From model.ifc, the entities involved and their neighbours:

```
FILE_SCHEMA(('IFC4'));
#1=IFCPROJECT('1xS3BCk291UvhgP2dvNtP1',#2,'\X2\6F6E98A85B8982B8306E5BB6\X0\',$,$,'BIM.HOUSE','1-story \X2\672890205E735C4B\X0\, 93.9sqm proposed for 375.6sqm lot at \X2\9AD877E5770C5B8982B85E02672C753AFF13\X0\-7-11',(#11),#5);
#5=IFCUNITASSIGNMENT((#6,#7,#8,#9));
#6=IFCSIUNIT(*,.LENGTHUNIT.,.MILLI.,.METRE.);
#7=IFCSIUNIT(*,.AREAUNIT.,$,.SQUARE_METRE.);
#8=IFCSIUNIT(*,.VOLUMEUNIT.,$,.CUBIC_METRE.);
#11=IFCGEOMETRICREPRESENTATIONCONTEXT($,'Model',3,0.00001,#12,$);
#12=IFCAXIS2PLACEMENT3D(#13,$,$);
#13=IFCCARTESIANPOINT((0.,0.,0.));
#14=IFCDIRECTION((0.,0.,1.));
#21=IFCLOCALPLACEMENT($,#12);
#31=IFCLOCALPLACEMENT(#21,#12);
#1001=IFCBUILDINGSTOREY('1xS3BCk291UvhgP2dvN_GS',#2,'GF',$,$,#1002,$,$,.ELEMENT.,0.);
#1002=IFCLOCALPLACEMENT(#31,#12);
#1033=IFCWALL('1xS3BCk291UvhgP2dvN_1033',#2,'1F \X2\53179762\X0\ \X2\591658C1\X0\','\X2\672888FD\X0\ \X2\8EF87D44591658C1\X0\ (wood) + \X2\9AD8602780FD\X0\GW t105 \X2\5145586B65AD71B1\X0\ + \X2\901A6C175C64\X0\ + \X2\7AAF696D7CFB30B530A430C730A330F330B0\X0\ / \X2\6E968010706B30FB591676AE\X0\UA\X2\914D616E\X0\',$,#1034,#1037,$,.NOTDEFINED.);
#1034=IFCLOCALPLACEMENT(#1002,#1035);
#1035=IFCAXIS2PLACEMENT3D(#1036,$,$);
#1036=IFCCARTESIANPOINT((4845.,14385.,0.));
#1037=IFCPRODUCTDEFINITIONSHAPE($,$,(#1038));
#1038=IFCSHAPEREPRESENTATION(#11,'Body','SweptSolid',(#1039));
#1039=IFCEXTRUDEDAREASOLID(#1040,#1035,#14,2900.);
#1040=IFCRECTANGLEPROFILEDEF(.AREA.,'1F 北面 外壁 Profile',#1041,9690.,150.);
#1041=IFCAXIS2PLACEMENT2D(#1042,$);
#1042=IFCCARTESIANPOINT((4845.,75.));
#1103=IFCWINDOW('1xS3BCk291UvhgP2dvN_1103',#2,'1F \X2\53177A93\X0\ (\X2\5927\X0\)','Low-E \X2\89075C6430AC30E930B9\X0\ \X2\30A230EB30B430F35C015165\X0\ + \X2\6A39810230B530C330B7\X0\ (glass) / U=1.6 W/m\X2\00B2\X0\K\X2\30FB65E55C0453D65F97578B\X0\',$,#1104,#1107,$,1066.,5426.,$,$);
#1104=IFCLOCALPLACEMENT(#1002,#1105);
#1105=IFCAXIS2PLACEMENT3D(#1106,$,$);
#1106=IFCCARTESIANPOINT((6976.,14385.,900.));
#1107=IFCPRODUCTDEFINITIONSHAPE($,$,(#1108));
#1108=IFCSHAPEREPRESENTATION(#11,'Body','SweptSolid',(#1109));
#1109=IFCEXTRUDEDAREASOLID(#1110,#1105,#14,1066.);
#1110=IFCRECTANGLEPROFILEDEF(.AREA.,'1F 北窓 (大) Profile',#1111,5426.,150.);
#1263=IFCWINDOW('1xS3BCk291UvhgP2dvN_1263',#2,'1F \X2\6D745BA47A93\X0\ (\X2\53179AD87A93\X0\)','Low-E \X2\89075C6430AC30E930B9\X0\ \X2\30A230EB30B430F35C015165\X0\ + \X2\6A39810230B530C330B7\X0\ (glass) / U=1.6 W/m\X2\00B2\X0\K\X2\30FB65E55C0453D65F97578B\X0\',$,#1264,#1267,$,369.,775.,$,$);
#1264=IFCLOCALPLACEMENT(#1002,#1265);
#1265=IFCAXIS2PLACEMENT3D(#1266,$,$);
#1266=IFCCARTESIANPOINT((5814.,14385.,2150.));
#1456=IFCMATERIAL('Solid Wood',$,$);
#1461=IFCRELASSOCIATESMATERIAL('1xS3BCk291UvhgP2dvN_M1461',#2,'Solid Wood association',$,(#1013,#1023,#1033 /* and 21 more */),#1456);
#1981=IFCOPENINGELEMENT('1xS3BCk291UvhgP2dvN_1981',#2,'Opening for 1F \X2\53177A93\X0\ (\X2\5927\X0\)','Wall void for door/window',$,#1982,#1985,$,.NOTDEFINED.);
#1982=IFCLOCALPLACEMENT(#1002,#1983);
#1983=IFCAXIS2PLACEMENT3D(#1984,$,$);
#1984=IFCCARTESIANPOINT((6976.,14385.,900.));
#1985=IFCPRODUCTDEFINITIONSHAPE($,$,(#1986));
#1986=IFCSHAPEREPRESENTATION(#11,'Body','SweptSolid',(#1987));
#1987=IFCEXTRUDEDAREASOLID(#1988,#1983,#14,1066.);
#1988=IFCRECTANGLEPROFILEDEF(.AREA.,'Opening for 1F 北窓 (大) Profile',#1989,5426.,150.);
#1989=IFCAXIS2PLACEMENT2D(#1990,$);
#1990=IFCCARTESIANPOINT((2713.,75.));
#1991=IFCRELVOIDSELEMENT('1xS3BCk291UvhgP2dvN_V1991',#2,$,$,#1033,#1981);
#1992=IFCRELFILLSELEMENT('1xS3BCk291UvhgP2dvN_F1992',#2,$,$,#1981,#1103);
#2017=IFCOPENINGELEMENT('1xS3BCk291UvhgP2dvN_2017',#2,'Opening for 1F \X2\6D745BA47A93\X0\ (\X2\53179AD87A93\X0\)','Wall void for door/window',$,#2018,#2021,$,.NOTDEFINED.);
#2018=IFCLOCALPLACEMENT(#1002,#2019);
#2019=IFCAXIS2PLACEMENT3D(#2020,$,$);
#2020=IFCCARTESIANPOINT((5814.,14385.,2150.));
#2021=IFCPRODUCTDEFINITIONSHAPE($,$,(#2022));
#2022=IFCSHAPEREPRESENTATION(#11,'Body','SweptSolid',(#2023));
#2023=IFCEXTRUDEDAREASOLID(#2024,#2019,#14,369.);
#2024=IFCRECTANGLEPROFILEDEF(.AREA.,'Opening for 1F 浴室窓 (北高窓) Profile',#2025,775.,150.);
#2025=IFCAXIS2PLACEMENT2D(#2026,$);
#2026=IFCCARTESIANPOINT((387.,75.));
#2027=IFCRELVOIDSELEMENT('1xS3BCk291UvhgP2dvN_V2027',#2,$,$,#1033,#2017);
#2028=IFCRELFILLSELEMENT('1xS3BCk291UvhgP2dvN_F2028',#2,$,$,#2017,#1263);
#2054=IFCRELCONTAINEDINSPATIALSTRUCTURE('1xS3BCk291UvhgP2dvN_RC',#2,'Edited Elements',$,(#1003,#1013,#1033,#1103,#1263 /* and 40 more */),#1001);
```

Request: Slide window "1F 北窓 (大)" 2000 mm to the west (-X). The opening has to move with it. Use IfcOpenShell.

```python
import ifcopenshell
import ifcopenshell.api.geometry
import ifcopenshell.util.placement

model = ifcopenshell.open("model.ifc")

window = model.by_guid("1xS3BCk291UvhgP2dvN_1103")
opening = window.FillsVoids[0].RelatingOpeningElement
wall = opening.VoidsElements[0].RelatingBuildingElement

wall_matrix = ifcopenshell.util.placement.get_local_placement(wall.ObjectPlacement)
shift = wall_matrix[:3, 0] * -2000.0
before = ifcopenshell.util.placement.get_local_placement(window.ObjectPlacement)[:3, 3].copy()

# The window is not placed relative to its opening, so move both.
for product in (opening, window):
    matrix = ifcopenshell.util.placement.get_local_placement(product.ObjectPlacement)
    matrix[:3, 3] += shift
    ifcopenshell.api.geometry.edit_object_placement(model, product=product, matrix=matrix, is_si=False)

after = ifcopenshell.util.placement.get_local_placement(window.ObjectPlacement)[:3, 3]
print("window moved by", (after - before).round(3) + 0.0)

model.write("model-out.ifc")
```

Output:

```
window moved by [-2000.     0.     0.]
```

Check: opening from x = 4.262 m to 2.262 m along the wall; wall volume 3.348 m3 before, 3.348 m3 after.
